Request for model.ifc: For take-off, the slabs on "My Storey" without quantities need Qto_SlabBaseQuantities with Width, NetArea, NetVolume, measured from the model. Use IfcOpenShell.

First a look at what the model holds.

```python
import ifcopenshell
import ifcopenshell.util.element
import ifcopenshell.util.unit

model = ifcopenshell.open("model.ifc")
print(model.schema)
for unit_type in ("LENGTHUNIT", "AREAUNIT", "VOLUMEUNIT"):
    print(unit_type, ifcopenshell.util.unit.calculate_unit_scale(model, unit_type))
storey = next(s for s in model.by_type("IfcBuildingStorey") if s.Name == "My Storey")
slabs = [e for e in ifcopenshell.util.element.get_decomposition(storey) if e.is_a("IfcSlab")]
for e in sorted(slabs, key=lambda e: e.id()):
    print(e.id(), e.is_a(), e.Name, list(ifcopenshell.util.element.get_psets(e, qtos_only=True)), sep=" | ")
```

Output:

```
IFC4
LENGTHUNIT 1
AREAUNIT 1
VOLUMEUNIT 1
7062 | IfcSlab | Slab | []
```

```python
import ifcopenshell
import ifcopenshell.api.pset
import ifcopenshell.geom
import ifcopenshell.util.element
import ifcopenshell.util.shape
import ifcopenshell.util.unit

model = ifcopenshell.open("model.ifc")
unit_scale = ifcopenshell.util.unit.calculate_unit_scale(model)
area_scale = ifcopenshell.util.unit.calculate_unit_scale(model, "AREAUNIT")
volume_scale = ifcopenshell.util.unit.calculate_unit_scale(model, "VOLUMEUNIT")
settings = ifcopenshell.geom.settings()

storey = next(s for s in model.by_type("IfcBuildingStorey") if s.Name == "My Storey")
slabs = [e for e in ifcopenshell.util.element.get_decomposition(storey) if e.is_a("IfcSlab")]

for e in sorted(slabs, key=lambda e: e.id()):
    if ifcopenshell.util.element.get_psets(e, qtos_only=True, should_inherit=False):
        continue
    # Geometry comes back in metres, in the element's own axes.
    shape = ifcopenshell.geom.create_shape(settings, e)
    values = {
        "Width": ifcopenshell.util.shape.get_z(shape.geometry) / unit_scale,
        "NetArea": ifcopenshell.util.shape.get_footprint_area(shape.geometry) / area_scale,
        "NetVolume": ifcopenshell.util.shape.get_volume(shape.geometry) / volume_scale,
    }
    qto = ifcopenshell.api.pset.add_qto(model, product=e, name="Qto_SlabBaseQuantities")
    ifcopenshell.api.pset.edit_qto(model, qto=qto, properties=values)
    print(e.id(), {k: round(v, 3) for k, v in values.items()})

model.write("model_updated.ifc")
```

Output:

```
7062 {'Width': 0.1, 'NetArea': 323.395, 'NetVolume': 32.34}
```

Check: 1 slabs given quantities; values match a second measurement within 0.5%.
